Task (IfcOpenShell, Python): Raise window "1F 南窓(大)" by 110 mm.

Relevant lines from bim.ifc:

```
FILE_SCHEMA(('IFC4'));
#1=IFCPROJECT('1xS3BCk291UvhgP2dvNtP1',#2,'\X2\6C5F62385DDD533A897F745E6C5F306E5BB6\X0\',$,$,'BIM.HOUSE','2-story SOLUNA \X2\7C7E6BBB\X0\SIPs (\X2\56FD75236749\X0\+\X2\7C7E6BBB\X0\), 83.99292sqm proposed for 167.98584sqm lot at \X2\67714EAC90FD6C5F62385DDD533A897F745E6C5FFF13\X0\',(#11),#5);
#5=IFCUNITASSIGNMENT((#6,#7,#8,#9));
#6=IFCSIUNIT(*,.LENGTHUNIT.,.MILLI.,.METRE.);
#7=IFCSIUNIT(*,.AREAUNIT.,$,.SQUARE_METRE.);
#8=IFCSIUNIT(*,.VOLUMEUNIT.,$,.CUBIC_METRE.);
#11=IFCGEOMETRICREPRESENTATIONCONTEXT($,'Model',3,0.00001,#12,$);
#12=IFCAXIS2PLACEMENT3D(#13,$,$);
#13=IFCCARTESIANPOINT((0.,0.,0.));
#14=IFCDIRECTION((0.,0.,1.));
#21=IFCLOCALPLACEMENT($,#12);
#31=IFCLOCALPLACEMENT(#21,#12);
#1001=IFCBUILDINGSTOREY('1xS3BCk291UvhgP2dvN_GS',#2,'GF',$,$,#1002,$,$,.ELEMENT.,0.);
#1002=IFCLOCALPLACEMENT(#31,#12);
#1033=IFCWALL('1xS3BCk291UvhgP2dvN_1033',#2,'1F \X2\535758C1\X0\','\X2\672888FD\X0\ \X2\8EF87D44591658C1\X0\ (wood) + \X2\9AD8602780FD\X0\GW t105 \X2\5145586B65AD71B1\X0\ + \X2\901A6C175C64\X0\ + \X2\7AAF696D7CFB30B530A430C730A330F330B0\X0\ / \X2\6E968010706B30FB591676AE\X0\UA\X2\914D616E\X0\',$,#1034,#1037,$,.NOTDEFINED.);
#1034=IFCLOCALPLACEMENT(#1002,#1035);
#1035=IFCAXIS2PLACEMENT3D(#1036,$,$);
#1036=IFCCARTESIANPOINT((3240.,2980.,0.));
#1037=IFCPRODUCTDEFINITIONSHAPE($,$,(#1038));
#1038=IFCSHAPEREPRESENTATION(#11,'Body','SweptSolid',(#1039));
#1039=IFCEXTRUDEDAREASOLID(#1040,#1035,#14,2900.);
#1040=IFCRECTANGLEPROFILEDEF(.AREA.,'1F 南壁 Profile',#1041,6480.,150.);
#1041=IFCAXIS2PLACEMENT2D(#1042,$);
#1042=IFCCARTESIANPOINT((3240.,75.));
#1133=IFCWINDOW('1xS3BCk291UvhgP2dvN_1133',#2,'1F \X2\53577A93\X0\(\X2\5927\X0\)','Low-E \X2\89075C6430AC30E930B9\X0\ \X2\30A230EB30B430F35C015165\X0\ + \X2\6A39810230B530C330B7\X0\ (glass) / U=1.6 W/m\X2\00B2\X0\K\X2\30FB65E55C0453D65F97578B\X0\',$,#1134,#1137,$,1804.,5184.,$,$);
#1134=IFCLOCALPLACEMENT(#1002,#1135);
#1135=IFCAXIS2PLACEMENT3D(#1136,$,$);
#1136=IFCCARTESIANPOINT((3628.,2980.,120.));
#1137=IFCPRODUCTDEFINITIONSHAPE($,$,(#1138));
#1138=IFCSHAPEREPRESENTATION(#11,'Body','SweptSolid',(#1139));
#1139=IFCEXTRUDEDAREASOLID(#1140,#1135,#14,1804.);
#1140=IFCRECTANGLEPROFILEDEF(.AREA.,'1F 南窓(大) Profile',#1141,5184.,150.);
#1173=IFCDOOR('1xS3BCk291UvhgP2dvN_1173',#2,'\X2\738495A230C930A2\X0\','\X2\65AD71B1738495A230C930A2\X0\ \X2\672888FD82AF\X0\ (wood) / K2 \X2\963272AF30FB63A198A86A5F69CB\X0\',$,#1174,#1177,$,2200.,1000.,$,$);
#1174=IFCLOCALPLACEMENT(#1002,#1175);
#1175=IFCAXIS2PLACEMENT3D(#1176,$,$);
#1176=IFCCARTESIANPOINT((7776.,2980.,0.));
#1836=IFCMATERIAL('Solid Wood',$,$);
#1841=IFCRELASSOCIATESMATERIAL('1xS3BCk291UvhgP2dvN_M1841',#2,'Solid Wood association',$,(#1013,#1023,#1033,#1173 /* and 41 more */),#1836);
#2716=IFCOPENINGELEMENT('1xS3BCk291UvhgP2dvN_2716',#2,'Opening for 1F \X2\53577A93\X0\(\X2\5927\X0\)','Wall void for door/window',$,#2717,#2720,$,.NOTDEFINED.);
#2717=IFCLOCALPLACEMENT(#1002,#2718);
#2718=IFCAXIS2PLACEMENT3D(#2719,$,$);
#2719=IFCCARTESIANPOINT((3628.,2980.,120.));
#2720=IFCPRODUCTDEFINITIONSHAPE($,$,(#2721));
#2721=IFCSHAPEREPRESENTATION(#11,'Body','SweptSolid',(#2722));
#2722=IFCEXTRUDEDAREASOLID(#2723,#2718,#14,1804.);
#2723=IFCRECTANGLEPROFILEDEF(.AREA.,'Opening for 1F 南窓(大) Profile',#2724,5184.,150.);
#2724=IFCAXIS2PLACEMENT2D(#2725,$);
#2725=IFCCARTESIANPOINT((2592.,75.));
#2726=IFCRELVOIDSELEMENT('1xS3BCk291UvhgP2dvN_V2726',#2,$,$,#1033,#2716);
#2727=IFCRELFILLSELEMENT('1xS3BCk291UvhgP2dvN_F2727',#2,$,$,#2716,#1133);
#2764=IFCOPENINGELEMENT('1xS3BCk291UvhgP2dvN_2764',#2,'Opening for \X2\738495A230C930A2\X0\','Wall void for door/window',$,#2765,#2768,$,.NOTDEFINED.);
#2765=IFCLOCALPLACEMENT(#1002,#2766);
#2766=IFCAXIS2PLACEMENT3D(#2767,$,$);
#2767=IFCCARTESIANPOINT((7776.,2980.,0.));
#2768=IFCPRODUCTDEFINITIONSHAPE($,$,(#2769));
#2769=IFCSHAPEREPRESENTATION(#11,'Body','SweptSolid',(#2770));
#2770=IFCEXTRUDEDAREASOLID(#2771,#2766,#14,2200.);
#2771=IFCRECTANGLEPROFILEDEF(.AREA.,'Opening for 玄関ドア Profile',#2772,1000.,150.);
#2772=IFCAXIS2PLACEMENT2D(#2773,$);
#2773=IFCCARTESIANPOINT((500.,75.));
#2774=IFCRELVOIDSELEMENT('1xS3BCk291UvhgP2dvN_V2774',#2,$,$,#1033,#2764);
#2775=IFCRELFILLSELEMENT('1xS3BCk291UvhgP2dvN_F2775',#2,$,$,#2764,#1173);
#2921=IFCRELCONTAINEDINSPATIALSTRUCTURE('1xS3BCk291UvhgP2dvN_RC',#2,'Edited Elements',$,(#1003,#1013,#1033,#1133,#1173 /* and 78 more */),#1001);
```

```python
import numpy as np
import ifcopenshell
import ifcopenshell.api.geometry
import ifcopenshell.util.placement
import ifcopenshell.util.unit

model = ifcopenshell.open("bim.ifc")
unit_scale = ifcopenshell.util.unit.calculate_unit_scale(model)

window = model.by_guid("1xS3BCk291UvhgP2dvN_1133")
opening = window.FillsVoids[0].RelatingOpeningElement
dz = 110.0

shift = np.array([0.0, 0.0, dz])
# The window is not placed relative to its opening, so move both.
for product in (opening, window):
    matrix = ifcopenshell.util.placement.get_local_placement(product.ObjectPlacement)
    matrix[:3, 3] += shift
    ifcopenshell.api.geometry.edit_object_placement(model, product=product, matrix=matrix, is_si=False)

print(f"moved by {dz * unit_scale:+.3f} m")

model.write("bim_updated.ifc")
```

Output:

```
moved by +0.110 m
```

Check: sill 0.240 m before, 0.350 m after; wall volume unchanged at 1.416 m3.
